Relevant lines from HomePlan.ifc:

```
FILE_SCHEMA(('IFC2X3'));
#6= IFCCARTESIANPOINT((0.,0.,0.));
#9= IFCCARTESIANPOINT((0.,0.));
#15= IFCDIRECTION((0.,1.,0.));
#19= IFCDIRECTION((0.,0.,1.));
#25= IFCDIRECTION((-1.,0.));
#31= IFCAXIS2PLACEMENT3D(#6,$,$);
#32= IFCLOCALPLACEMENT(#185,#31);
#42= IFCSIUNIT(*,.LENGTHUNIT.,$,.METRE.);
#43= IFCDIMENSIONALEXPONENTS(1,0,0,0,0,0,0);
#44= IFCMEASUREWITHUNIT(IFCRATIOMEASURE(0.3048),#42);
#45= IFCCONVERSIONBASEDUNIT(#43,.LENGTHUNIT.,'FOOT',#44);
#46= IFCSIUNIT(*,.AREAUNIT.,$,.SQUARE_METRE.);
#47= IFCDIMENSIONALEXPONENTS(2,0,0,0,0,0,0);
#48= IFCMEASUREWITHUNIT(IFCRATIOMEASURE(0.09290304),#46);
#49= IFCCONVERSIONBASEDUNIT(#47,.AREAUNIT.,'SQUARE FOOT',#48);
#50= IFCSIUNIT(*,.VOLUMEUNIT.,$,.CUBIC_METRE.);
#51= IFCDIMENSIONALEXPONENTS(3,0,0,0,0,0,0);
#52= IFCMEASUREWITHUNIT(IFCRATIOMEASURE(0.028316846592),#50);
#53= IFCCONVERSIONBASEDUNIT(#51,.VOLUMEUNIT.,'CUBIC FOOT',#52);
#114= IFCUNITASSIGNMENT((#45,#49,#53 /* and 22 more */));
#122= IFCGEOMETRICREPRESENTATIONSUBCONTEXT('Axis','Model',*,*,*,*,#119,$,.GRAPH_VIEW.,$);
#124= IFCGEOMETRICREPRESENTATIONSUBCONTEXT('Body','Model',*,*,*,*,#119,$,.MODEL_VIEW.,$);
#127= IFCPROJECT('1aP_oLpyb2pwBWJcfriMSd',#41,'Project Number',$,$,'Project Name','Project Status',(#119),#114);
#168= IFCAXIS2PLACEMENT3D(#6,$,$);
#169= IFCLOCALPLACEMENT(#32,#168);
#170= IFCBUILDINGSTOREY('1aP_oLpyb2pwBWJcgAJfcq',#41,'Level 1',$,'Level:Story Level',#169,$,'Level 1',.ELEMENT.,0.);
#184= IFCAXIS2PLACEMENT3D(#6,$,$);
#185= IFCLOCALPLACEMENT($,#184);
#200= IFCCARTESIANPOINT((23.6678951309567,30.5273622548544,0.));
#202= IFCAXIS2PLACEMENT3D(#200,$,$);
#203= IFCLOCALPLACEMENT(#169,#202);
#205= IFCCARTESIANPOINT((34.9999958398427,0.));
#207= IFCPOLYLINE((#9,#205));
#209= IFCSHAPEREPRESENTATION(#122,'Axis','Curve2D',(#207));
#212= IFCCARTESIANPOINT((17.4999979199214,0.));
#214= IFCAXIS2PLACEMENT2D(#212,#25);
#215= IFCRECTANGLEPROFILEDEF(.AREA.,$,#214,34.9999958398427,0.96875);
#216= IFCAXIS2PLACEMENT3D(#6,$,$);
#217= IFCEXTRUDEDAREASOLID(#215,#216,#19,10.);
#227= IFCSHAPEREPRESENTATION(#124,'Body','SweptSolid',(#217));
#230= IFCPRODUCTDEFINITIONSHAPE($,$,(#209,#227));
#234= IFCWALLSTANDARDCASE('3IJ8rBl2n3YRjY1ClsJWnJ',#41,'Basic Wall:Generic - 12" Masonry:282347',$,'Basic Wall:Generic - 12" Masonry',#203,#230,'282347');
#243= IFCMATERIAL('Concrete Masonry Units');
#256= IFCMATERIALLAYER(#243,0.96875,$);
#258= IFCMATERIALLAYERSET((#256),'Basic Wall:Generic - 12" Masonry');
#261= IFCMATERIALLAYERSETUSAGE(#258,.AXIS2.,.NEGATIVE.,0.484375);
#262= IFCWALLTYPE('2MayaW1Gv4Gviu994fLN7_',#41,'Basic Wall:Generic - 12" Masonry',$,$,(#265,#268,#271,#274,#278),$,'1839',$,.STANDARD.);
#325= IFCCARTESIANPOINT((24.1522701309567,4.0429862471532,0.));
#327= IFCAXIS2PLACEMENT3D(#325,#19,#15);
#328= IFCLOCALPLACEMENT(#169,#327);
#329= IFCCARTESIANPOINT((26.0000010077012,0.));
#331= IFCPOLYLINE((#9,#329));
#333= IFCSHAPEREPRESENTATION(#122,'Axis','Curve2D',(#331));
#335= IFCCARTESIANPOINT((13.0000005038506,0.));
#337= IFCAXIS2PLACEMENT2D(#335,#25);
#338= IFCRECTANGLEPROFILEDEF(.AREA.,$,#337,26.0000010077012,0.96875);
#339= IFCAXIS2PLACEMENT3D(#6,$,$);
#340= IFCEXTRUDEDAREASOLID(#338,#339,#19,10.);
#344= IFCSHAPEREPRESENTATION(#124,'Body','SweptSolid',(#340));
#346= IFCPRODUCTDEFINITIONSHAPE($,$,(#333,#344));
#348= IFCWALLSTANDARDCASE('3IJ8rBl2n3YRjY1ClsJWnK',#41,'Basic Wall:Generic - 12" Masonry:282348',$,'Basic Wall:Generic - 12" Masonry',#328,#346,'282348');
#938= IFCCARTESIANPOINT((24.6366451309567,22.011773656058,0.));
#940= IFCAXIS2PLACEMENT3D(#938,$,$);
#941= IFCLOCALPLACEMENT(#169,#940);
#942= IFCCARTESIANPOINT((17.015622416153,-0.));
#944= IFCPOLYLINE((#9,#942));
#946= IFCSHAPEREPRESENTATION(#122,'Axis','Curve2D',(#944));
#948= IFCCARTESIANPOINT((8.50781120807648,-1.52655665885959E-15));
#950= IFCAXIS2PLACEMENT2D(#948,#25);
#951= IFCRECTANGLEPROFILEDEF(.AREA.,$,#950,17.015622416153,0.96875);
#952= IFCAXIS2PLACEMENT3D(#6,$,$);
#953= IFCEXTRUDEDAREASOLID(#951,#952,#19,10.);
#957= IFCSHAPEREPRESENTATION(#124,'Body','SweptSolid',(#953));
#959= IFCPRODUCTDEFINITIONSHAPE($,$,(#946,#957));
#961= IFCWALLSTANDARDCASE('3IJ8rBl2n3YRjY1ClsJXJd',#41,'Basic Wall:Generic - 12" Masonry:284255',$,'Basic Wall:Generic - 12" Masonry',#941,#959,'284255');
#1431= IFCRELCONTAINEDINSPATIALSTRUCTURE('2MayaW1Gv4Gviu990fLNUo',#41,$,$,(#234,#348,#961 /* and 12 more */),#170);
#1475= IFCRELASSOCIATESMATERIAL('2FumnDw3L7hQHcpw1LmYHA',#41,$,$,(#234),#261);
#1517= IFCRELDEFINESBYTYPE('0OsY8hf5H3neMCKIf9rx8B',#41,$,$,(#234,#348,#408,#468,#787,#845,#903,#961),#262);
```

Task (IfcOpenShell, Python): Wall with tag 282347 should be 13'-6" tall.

```python
import ifcopenshell
import ifcopenshell.geom
import ifcopenshell.util.representation
import ifcopenshell.util.shape
import ifcopenshell.util.unit

model = ifcopenshell.open("HomePlan.ifc")
unit_scale = ifcopenshell.util.unit.calculate_unit_scale(model)
settings = ifcopenshell.geom.settings()


def volume(element):
    """Net volume in cubic metres, openings subtracted."""
    shape = ifcopenshell.geom.create_shape(settings, element)
    return ifcopenshell.util.shape.get_volume(shape.geometry)


wall = model.by_id(234)
before = volume(wall)

body = ifcopenshell.util.representation.get_representation(wall, "Model", "Body")
solid = body.Items[0]
old_height = solid.Depth
solid.Depth = 162 * 0.0254 / unit_scale
after = volume(wall)

print(f"height {old_height:g} -> {solid.Depth:g}, volume {before:.3f} -> {after:.3f} m3")

model.write("HomePlan_updated.ifc")
```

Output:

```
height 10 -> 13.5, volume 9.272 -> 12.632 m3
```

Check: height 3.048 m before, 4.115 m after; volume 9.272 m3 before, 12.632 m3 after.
